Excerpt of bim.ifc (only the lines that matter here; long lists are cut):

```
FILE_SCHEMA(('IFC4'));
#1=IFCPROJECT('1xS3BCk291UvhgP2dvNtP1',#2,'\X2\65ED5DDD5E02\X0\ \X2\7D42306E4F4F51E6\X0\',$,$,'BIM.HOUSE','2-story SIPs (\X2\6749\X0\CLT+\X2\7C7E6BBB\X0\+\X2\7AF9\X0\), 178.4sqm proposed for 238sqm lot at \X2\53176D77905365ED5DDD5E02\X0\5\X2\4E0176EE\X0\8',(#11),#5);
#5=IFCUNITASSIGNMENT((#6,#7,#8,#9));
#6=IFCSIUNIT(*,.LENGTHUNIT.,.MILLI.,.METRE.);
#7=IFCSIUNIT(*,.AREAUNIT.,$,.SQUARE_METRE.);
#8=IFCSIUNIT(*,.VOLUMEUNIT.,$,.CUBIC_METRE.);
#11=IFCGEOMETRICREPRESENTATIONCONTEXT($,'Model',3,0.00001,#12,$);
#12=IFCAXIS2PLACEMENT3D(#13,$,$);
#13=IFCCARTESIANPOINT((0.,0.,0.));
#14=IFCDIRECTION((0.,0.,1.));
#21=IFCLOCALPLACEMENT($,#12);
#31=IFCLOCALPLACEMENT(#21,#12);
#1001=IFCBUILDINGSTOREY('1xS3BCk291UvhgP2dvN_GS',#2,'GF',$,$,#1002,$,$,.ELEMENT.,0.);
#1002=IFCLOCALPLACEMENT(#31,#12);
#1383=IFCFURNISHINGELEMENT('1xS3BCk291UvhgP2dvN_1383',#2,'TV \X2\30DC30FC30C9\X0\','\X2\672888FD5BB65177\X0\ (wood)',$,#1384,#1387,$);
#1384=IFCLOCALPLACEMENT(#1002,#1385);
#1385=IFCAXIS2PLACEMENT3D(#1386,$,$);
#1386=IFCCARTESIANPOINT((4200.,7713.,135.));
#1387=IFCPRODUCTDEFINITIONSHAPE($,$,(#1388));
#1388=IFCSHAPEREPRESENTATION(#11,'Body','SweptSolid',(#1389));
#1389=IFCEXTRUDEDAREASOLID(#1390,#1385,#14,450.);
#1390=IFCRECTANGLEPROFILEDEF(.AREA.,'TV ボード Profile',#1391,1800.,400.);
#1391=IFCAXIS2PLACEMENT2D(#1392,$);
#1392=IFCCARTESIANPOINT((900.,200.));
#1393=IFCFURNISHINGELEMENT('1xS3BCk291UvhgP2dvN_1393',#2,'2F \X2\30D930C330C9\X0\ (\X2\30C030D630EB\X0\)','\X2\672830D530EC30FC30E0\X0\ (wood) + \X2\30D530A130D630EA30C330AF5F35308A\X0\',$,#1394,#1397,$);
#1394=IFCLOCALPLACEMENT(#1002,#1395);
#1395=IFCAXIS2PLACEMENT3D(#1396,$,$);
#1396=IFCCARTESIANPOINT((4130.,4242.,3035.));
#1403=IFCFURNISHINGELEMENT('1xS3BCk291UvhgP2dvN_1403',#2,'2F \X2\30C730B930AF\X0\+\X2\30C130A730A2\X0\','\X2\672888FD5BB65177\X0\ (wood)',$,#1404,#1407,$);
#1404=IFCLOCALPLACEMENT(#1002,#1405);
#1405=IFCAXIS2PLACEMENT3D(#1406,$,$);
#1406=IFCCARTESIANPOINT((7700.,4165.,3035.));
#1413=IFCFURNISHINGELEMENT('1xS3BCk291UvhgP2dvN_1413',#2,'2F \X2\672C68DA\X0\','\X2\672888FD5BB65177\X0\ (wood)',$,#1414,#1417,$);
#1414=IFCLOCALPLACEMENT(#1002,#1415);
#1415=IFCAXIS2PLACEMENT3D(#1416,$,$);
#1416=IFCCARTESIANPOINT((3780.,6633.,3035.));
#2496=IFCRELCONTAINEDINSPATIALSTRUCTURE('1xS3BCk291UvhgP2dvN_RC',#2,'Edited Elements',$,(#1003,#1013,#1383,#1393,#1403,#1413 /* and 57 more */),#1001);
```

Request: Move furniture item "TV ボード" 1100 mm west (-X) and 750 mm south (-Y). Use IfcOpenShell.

```python
import ifcopenshell
import ifcopenshell.api.geometry
import ifcopenshell.util.placement
import ifcopenshell.util.unit

model = ifcopenshell.open("bim.ifc")
unit_scale = ifcopenshell.util.unit.calculate_unit_scale(model)

item = model.by_guid("1xS3BCk291UvhgP2dvN_1383")
matrix = ifcopenshell.util.placement.get_local_placement(item.ObjectPlacement)
matrix[0, 3] -= 1.1 / unit_scale
matrix[1, 3] -= 0.75 / unit_scale
ifcopenshell.api.geometry.edit_object_placement(model, product=item, matrix=matrix, is_si=False)

print(ifcopenshell.util.placement.get_local_placement(item.ObjectPlacement).round(3) + 0.0)

model.write("bim-out.ifc")
```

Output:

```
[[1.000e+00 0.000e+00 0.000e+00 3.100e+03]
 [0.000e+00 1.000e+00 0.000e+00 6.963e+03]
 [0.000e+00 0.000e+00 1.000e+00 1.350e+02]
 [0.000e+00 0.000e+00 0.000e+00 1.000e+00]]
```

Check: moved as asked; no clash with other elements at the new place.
